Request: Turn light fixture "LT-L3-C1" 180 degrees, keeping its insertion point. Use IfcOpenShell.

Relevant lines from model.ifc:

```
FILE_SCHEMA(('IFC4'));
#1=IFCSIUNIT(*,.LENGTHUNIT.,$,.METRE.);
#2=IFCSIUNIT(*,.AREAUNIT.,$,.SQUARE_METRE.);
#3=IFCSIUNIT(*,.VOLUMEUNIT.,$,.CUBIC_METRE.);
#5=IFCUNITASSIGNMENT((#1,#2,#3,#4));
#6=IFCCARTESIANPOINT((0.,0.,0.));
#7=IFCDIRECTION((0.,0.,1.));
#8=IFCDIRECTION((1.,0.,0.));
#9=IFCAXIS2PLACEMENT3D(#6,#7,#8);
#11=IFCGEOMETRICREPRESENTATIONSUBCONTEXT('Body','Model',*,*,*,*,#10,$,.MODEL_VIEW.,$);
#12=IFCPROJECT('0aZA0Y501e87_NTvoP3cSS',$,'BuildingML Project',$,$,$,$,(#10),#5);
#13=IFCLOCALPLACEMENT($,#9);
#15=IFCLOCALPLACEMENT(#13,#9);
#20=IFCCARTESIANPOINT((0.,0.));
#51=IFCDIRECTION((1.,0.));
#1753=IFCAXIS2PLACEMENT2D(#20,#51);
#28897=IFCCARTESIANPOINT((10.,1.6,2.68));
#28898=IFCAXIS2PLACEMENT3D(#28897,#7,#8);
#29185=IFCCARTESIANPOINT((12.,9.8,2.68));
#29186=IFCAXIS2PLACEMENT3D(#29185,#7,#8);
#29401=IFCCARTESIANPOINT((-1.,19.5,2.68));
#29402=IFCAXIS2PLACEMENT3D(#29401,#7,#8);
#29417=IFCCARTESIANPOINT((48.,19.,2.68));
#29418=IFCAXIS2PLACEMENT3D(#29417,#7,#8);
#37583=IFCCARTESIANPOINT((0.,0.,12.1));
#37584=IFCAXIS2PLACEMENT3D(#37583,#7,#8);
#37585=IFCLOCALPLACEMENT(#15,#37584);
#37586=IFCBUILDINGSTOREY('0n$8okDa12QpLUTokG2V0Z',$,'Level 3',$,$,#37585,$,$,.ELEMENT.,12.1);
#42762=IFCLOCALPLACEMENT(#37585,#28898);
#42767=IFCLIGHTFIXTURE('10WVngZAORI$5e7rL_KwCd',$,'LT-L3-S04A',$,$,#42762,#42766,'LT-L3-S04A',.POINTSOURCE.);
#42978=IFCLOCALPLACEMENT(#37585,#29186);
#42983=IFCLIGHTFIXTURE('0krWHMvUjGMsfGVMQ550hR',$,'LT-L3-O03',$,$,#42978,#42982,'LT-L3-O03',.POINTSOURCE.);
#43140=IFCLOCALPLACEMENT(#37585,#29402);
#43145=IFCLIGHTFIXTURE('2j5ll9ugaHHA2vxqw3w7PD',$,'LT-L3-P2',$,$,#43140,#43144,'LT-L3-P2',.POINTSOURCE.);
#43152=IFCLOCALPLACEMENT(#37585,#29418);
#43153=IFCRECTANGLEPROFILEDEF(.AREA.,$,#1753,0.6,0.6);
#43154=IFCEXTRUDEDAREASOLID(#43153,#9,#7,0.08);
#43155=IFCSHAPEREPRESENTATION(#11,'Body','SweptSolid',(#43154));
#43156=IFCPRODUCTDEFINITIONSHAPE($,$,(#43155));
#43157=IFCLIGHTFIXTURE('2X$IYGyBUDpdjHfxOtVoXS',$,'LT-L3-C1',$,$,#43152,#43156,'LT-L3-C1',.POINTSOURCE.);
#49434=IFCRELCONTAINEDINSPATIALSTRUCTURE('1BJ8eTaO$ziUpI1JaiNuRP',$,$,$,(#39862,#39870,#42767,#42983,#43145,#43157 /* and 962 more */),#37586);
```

```python
import ifcopenshell
import ifcopenshell.api.geometry
import ifcopenshell.util.placement

model = ifcopenshell.open("model.ifc")

item = model.by_guid("2X$IYGyBUDpdjHfxOtVoXS")
matrix = ifcopenshell.util.placement.get_local_placement(item.ObjectPlacement)
matrix = matrix @ ifcopenshell.util.placement.rotation(180, "Z")
ifcopenshell.api.geometry.edit_object_placement(model, product=item, matrix=matrix, is_si=False)

print(ifcopenshell.util.placement.get_local_placement(item.ObjectPlacement).round(3) + 0.0)

model.write("model_rev.ifc")
```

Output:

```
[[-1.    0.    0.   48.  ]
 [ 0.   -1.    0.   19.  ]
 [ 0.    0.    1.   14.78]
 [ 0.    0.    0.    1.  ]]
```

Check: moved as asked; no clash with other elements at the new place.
